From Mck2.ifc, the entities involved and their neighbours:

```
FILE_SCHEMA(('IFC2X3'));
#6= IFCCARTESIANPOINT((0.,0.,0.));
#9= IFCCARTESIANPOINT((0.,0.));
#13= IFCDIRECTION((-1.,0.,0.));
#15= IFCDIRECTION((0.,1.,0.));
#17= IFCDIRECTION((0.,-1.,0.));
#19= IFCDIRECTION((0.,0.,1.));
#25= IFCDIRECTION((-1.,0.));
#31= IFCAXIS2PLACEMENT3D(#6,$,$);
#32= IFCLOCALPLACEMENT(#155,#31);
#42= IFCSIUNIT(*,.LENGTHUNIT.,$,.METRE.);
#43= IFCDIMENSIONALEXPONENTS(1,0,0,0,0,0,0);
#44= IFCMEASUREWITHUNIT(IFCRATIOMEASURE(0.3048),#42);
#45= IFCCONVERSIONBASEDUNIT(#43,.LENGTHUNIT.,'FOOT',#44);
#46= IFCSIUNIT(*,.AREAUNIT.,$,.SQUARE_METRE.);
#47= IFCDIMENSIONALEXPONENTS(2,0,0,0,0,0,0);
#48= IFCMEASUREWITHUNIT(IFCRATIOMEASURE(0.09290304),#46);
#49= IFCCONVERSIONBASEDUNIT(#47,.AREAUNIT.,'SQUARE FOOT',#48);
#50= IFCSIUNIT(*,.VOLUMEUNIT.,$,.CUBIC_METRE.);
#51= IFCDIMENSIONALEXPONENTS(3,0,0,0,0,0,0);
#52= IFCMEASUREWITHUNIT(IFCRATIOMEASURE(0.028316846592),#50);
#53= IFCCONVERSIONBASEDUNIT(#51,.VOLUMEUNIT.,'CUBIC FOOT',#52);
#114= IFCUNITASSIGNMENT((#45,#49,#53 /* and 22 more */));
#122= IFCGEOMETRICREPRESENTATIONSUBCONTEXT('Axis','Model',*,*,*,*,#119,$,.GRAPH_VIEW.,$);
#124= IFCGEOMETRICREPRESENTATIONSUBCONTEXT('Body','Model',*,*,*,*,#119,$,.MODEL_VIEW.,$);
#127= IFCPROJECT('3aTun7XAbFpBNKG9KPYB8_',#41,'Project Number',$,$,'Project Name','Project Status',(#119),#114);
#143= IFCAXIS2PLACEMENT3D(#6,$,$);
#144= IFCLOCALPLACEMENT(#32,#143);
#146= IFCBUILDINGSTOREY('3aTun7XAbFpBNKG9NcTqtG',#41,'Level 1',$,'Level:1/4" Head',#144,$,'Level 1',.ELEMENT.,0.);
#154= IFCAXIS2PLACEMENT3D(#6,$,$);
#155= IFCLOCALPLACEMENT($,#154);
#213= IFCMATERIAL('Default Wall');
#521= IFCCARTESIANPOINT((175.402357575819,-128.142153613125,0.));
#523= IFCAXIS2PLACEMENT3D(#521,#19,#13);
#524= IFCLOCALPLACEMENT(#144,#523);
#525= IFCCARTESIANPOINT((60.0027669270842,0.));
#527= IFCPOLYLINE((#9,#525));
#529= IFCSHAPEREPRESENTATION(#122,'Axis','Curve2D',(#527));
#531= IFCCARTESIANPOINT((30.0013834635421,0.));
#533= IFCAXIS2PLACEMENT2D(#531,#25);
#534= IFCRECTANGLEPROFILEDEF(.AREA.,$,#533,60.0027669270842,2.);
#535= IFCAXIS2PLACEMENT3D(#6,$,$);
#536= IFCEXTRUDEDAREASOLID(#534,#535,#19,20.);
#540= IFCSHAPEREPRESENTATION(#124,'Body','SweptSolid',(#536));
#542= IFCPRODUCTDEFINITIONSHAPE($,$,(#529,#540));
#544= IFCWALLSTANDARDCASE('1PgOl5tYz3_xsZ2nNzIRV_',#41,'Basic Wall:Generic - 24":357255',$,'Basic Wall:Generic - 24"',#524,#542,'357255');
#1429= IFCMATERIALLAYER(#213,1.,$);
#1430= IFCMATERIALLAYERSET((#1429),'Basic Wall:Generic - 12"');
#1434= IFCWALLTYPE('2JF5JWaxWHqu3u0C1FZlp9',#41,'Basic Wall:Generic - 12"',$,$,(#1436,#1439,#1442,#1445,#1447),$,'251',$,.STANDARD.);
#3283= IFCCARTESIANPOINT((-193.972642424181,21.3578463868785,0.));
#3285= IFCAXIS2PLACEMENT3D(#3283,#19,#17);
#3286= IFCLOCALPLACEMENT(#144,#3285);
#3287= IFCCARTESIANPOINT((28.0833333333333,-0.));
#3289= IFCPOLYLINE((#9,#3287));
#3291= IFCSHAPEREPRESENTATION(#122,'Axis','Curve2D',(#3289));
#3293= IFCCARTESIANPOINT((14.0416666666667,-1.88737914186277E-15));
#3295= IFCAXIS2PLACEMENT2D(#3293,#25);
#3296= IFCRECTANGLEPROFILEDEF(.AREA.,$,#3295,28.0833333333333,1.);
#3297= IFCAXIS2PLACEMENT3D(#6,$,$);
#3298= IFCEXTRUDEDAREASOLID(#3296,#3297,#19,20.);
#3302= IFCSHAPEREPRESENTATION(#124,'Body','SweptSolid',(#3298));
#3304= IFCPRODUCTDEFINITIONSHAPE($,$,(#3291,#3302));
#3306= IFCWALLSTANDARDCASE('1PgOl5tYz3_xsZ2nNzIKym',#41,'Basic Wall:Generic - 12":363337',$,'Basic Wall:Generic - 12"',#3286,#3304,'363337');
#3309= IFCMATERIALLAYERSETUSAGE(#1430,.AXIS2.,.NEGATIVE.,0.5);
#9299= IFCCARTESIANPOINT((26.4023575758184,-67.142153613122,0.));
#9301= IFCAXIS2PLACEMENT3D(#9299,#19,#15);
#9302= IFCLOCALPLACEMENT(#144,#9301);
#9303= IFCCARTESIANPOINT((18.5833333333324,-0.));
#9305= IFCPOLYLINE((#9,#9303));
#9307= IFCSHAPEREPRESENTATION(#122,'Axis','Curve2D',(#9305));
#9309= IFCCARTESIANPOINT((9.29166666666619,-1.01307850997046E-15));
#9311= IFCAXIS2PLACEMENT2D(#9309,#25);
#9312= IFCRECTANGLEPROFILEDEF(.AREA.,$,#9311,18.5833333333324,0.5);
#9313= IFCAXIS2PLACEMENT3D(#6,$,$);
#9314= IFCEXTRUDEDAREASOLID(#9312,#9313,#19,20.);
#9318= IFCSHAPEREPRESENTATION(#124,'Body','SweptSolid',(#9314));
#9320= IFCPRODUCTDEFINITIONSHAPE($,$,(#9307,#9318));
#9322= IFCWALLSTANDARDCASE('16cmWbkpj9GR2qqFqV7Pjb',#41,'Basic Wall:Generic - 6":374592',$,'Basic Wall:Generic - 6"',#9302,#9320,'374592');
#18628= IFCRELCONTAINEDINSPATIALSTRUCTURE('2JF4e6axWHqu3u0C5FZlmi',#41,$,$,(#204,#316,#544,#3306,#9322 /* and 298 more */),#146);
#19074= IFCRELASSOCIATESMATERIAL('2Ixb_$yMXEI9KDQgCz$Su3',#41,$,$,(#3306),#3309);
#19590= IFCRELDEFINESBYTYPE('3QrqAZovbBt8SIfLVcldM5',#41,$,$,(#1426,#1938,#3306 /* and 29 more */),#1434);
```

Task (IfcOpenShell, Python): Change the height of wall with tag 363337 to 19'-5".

```python
import ifcopenshell
import ifcopenshell.geom
import ifcopenshell.util.representation
import ifcopenshell.util.shape
import ifcopenshell.util.unit

model = ifcopenshell.open("Mck2.ifc")
unit_scale = ifcopenshell.util.unit.calculate_unit_scale(model)
settings = ifcopenshell.geom.settings()


def volume(element):
    """Net volume in cubic metres, openings subtracted."""
    shape = ifcopenshell.geom.create_shape(settings, element)
    return ifcopenshell.util.shape.get_volume(shape.geometry)


wall = model.by_guid("1PgOl5tYz3_xsZ2nNzIKym")
before = volume(wall)

body = ifcopenshell.util.representation.get_representation(wall, "Model", "Body")
solid = body.Items[0]
old_height = solid.Depth
solid.Depth = 233 * 0.0254 / unit_scale
after = volume(wall)

print(f"height {old_height:g} -> {solid.Depth:g}, volume {before:.3f} -> {after:.3f} m3")

model.write("Mck2_updated.ifc")
```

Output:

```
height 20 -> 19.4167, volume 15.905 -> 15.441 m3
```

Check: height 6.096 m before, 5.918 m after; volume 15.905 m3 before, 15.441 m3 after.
